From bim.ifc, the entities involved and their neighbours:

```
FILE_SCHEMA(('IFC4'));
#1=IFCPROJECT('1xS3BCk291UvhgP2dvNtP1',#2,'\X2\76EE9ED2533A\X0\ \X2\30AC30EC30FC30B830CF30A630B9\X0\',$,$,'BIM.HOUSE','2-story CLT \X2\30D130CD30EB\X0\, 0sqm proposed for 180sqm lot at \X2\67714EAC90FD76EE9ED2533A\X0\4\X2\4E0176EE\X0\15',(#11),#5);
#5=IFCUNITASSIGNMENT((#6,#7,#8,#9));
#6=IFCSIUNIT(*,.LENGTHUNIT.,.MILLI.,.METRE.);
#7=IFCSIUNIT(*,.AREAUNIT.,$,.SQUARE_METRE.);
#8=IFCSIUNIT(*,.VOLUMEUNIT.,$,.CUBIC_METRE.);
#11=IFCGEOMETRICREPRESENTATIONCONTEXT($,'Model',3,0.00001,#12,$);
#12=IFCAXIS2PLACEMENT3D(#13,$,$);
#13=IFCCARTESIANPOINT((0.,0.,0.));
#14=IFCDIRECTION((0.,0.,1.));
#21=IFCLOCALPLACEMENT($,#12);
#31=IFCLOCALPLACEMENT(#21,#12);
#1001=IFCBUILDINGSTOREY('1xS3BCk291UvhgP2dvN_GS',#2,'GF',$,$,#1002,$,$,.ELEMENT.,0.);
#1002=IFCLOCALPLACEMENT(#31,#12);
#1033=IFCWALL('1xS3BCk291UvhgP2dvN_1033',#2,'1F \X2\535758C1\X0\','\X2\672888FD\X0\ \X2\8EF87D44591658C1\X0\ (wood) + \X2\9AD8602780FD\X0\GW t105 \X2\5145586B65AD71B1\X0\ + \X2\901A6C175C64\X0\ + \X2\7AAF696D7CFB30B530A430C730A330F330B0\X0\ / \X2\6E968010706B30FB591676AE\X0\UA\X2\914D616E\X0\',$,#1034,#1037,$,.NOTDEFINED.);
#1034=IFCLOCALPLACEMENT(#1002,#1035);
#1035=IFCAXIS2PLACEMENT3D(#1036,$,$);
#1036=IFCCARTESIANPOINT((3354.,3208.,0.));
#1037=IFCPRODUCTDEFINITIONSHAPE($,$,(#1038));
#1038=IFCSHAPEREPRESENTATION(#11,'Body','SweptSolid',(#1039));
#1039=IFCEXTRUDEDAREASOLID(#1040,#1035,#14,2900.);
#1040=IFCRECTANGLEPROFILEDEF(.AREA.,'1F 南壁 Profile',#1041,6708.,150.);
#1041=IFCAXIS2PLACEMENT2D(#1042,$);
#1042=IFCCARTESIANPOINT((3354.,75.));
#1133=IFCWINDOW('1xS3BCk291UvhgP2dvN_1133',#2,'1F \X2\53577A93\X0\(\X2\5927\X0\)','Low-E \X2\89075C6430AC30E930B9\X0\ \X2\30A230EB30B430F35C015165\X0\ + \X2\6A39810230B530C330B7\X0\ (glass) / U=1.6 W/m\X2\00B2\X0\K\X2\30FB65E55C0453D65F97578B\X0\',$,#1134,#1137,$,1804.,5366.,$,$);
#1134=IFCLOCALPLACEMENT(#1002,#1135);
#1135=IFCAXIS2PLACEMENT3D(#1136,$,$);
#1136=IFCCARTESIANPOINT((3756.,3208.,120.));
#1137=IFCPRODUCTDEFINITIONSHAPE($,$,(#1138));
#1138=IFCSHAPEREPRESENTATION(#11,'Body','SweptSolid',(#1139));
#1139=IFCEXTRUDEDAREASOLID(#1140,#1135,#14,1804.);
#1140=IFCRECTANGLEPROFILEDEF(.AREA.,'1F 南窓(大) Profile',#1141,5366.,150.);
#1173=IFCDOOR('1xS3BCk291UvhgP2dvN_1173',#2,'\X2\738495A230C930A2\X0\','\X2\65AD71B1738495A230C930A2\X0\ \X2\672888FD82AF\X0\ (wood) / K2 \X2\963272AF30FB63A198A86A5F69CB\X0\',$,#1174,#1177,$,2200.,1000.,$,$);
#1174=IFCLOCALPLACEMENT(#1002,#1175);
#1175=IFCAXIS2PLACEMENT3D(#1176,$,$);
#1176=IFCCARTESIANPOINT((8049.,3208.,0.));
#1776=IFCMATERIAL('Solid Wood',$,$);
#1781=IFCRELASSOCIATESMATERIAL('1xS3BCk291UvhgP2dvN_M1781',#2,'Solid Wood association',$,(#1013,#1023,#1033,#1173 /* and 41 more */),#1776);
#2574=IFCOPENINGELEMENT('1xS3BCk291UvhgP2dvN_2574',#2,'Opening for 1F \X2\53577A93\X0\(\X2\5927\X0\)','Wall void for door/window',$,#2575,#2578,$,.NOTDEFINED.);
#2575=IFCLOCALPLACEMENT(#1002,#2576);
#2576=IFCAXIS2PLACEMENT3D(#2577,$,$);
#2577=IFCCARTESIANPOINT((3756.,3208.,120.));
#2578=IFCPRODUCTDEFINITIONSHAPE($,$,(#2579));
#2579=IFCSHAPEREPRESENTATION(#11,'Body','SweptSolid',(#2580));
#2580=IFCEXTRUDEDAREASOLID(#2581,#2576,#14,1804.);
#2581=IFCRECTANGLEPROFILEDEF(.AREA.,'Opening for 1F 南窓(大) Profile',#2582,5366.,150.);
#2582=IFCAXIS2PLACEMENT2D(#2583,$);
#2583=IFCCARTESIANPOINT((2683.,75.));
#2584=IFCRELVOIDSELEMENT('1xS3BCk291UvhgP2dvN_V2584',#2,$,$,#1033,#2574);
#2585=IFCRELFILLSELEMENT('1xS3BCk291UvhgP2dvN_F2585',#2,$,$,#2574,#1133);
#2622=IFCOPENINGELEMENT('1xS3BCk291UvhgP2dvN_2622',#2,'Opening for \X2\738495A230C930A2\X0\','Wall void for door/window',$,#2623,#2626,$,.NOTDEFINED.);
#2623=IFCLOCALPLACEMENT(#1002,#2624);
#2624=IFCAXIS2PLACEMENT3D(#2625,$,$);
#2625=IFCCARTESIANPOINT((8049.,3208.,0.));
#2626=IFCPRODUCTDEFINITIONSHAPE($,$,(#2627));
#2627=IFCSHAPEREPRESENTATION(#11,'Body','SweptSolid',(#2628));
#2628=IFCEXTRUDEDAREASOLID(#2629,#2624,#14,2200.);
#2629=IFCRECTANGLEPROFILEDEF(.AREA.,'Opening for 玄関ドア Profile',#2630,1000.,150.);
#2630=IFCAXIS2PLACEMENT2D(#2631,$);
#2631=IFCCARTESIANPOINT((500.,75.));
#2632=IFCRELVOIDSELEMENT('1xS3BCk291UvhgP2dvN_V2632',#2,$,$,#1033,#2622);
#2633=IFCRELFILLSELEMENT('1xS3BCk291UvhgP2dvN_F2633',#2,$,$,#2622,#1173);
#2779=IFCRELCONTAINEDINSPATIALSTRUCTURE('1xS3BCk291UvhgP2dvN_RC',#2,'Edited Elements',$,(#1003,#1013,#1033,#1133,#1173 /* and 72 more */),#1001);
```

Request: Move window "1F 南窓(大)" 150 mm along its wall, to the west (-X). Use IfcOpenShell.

```python
import ifcopenshell
import ifcopenshell.api.geometry
import ifcopenshell.util.placement
import ifcopenshell.util.unit

model = ifcopenshell.open("bim.ifc")
unit_scale = ifcopenshell.util.unit.calculate_unit_scale(model)

window = model.by_guid("1xS3BCk291UvhgP2dvN_1133")
opening = window.FillsVoids[0].RelatingOpeningElement
wall = opening.VoidsElements[0].RelatingBuildingElement

wall_matrix = ifcopenshell.util.placement.get_local_placement(wall.ObjectPlacement)
shift = wall_matrix[:3, 0] * -0.15 / unit_scale
before = ifcopenshell.util.placement.get_local_placement(window.ObjectPlacement)[:3, 3].copy()

# The window is not placed relative to its opening, so move both.
for product in (opening, window):
    matrix = ifcopenshell.util.placement.get_local_placement(product.ObjectPlacement)
    matrix[:3, 3] += shift
    ifcopenshell.api.geometry.edit_object_placement(model, product=product, matrix=matrix, is_si=False)

after = ifcopenshell.util.placement.get_local_placement(window.ObjectPlacement)[:3, 3]
print("window moved by", (after - before).round(3) + 0.0)

model.write("bim_v2.ifc")
```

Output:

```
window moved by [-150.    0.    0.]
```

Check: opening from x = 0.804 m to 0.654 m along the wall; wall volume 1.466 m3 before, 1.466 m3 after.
